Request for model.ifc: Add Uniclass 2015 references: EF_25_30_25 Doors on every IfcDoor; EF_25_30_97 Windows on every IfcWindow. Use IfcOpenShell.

First a look at what the model holds.

```python
import ifcopenshell

model = ifcopenshell.open("model.ifc")
print(model.schema)
print("classifications:", [c.Name for c in model.by_type("IfcClassification")])
for ifc_class in ("IfcDoor", "IfcRoof", "IfcStair", "IfcWall", "IfcWindow"):
    print(ifc_class, len(model.by_type(ifc_class)))
```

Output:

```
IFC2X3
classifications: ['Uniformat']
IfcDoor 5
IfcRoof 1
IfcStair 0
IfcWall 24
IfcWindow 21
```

```python
import ifcopenshell
import ifcopenshell.api.classification

model = ifcopenshell.open("model.ifc")

# IFC2X3 requires Source and Edition and has no link from the project to the system.
system = model.create_entity("IfcClassification", Source="NBS", Edition="2015", Name="Uniclass 2015")

codes = {
    "IfcDoor": ("EF_25_30_25", "Doors"),
    "IfcWindow": ("EF_25_30_97", "Windows"),
}
for ifc_class, (code, name) in codes.items():
    products = model.by_type(ifc_class)
    ifcopenshell.api.classification.add_reference(
        model, products=products, classification=system, identification=code, name=name
    )
    print(code, len(products))

model.write("model_rev.ifc")
```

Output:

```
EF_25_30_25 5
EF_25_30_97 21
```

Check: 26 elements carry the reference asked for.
